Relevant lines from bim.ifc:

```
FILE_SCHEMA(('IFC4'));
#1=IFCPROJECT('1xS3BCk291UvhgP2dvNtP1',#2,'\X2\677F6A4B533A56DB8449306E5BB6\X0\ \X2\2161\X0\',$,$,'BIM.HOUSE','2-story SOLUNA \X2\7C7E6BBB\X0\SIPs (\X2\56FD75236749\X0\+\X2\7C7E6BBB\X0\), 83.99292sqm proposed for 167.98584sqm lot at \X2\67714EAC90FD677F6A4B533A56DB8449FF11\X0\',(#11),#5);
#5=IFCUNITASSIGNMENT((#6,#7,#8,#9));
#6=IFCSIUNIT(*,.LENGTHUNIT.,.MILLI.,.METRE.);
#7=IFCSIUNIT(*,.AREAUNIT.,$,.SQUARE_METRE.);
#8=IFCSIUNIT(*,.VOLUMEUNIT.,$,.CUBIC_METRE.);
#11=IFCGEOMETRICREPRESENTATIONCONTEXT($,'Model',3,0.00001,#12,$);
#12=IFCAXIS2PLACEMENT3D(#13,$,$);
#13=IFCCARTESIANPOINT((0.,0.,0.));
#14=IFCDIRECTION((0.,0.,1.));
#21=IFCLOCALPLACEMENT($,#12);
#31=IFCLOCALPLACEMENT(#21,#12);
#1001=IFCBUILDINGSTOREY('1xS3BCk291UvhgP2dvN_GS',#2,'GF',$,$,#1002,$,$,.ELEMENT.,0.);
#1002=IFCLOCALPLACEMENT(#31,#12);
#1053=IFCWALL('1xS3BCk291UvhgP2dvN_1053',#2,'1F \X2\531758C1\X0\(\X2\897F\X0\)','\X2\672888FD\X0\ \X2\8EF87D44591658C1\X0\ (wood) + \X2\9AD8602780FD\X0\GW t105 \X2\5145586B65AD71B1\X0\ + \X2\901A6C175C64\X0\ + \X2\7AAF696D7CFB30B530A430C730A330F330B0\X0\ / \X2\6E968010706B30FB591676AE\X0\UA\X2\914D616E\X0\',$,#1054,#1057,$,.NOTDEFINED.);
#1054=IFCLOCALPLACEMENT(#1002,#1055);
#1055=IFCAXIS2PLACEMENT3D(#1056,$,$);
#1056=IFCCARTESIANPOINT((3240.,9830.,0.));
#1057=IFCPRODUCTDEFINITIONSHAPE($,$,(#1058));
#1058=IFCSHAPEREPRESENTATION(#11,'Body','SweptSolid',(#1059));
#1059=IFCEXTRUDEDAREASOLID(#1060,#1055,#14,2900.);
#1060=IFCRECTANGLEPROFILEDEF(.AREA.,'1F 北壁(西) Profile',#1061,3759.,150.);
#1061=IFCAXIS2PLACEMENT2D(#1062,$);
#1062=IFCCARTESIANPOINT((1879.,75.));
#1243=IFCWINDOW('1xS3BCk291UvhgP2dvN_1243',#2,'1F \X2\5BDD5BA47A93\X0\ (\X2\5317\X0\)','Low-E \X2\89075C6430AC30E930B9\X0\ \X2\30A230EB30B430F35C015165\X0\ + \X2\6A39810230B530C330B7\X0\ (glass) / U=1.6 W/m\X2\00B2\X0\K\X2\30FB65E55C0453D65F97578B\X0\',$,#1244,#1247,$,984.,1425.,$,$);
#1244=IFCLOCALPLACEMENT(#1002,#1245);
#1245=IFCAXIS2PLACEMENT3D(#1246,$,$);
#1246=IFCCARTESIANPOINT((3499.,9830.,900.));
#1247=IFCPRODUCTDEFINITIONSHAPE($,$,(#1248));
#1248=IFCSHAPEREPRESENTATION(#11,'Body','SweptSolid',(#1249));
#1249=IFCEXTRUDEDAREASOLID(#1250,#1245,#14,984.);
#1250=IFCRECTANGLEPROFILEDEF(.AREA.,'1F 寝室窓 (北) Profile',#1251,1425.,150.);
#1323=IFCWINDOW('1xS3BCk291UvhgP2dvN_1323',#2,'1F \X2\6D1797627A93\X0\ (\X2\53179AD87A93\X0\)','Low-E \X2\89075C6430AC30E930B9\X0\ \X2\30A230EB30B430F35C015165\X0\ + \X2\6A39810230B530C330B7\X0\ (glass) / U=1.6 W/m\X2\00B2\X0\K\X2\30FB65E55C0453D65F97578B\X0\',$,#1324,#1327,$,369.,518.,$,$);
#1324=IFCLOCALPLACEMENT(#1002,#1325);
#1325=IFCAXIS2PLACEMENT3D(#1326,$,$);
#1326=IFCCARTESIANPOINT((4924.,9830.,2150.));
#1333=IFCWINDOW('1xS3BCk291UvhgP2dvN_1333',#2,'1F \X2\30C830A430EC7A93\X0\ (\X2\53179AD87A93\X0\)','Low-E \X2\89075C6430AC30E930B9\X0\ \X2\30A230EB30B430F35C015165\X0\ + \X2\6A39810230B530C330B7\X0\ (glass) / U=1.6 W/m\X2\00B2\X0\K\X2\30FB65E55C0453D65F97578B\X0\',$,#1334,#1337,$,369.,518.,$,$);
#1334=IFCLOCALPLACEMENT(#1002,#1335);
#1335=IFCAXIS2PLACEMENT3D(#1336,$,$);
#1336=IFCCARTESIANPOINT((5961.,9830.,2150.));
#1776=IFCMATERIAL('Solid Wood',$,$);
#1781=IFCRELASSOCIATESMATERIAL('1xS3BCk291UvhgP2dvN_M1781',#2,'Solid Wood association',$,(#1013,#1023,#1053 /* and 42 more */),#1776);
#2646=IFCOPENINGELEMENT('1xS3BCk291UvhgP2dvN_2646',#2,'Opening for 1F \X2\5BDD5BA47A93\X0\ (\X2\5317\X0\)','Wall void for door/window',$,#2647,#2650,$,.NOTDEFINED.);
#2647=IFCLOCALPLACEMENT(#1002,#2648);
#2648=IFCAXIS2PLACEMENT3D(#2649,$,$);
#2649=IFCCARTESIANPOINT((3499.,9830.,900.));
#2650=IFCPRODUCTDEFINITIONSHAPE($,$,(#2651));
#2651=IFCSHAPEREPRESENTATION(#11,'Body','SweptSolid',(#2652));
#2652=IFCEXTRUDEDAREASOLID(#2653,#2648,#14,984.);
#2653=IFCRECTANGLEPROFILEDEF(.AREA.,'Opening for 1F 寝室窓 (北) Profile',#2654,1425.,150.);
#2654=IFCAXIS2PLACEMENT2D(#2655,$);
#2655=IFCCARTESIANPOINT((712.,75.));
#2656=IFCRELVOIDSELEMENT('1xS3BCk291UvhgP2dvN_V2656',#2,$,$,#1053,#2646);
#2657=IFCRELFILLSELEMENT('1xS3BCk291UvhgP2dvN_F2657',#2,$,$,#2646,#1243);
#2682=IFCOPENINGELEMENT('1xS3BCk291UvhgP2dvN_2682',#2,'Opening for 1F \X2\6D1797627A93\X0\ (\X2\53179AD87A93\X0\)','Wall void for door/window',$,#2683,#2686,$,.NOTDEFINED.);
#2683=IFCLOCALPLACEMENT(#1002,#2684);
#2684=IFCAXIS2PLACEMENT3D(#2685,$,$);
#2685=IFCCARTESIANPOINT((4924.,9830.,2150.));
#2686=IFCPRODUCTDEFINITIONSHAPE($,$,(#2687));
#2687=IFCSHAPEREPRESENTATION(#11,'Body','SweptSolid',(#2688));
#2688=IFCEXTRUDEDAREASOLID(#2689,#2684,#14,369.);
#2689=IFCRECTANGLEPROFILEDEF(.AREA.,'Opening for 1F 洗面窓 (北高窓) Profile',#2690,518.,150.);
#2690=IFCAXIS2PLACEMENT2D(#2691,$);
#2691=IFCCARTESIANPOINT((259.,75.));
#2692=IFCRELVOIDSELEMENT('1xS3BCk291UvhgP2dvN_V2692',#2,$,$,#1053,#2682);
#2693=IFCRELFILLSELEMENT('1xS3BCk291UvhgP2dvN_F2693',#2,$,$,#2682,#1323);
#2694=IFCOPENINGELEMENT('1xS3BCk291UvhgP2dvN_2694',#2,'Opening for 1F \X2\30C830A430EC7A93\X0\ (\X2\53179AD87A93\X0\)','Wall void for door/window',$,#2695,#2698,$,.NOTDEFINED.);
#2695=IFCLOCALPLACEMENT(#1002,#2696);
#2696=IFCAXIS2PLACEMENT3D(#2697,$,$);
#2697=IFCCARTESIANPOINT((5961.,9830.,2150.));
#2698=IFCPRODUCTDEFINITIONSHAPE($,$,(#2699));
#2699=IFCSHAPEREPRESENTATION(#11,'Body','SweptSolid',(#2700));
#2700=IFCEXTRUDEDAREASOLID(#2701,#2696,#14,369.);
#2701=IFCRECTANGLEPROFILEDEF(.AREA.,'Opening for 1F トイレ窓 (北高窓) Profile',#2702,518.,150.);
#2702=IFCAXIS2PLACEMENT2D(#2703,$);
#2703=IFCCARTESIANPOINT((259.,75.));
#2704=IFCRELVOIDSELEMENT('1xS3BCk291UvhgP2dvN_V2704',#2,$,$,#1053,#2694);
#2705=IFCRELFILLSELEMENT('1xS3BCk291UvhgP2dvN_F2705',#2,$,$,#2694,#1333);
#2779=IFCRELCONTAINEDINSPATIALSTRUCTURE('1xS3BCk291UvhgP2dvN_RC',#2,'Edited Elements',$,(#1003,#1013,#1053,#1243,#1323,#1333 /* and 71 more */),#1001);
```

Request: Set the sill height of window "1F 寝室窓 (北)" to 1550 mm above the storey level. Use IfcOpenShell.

```python
import numpy as np
import ifcopenshell
import ifcopenshell.api.geometry
import ifcopenshell.geom
import ifcopenshell.util.element
import ifcopenshell.util.placement
import ifcopenshell.util.shape
import ifcopenshell.util.unit

model = ifcopenshell.open("bim.ifc")
unit_scale = ifcopenshell.util.unit.calculate_unit_scale(model)

window = model.by_id(1243)
opening = window.FillsVoids[0].RelatingOpeningElement
storey = ifcopenshell.util.element.get_container(window, ifc_class="IfcBuildingStorey")
level = ifcopenshell.util.placement.get_local_placement(storey.ObjectPlacement)[2, 3]

# The opening's origin need not be at the sill, so measure its lowest point.
shape = ifcopenshell.geom.create_shape(ifcopenshell.geom.settings(), opening)
bottom = ifcopenshell.util.shape.get_shape_bottom_elevation(shape, shape.geometry) / unit_scale
dz = level + 1.55 / unit_scale - bottom

shift = np.array([0.0, 0.0, dz])
# The window is not placed relative to its opening, so move both.
for product in (opening, window):
    matrix = ifcopenshell.util.placement.get_local_placement(product.ObjectPlacement)
    matrix[:3, 3] += shift
    ifcopenshell.api.geometry.edit_object_placement(model, product=product, matrix=matrix, is_si=False)

print(f"moved by {dz * unit_scale:+.3f} m")

model.write("bim_edited.ifc")
```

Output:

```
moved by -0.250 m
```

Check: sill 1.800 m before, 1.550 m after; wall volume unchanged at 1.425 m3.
